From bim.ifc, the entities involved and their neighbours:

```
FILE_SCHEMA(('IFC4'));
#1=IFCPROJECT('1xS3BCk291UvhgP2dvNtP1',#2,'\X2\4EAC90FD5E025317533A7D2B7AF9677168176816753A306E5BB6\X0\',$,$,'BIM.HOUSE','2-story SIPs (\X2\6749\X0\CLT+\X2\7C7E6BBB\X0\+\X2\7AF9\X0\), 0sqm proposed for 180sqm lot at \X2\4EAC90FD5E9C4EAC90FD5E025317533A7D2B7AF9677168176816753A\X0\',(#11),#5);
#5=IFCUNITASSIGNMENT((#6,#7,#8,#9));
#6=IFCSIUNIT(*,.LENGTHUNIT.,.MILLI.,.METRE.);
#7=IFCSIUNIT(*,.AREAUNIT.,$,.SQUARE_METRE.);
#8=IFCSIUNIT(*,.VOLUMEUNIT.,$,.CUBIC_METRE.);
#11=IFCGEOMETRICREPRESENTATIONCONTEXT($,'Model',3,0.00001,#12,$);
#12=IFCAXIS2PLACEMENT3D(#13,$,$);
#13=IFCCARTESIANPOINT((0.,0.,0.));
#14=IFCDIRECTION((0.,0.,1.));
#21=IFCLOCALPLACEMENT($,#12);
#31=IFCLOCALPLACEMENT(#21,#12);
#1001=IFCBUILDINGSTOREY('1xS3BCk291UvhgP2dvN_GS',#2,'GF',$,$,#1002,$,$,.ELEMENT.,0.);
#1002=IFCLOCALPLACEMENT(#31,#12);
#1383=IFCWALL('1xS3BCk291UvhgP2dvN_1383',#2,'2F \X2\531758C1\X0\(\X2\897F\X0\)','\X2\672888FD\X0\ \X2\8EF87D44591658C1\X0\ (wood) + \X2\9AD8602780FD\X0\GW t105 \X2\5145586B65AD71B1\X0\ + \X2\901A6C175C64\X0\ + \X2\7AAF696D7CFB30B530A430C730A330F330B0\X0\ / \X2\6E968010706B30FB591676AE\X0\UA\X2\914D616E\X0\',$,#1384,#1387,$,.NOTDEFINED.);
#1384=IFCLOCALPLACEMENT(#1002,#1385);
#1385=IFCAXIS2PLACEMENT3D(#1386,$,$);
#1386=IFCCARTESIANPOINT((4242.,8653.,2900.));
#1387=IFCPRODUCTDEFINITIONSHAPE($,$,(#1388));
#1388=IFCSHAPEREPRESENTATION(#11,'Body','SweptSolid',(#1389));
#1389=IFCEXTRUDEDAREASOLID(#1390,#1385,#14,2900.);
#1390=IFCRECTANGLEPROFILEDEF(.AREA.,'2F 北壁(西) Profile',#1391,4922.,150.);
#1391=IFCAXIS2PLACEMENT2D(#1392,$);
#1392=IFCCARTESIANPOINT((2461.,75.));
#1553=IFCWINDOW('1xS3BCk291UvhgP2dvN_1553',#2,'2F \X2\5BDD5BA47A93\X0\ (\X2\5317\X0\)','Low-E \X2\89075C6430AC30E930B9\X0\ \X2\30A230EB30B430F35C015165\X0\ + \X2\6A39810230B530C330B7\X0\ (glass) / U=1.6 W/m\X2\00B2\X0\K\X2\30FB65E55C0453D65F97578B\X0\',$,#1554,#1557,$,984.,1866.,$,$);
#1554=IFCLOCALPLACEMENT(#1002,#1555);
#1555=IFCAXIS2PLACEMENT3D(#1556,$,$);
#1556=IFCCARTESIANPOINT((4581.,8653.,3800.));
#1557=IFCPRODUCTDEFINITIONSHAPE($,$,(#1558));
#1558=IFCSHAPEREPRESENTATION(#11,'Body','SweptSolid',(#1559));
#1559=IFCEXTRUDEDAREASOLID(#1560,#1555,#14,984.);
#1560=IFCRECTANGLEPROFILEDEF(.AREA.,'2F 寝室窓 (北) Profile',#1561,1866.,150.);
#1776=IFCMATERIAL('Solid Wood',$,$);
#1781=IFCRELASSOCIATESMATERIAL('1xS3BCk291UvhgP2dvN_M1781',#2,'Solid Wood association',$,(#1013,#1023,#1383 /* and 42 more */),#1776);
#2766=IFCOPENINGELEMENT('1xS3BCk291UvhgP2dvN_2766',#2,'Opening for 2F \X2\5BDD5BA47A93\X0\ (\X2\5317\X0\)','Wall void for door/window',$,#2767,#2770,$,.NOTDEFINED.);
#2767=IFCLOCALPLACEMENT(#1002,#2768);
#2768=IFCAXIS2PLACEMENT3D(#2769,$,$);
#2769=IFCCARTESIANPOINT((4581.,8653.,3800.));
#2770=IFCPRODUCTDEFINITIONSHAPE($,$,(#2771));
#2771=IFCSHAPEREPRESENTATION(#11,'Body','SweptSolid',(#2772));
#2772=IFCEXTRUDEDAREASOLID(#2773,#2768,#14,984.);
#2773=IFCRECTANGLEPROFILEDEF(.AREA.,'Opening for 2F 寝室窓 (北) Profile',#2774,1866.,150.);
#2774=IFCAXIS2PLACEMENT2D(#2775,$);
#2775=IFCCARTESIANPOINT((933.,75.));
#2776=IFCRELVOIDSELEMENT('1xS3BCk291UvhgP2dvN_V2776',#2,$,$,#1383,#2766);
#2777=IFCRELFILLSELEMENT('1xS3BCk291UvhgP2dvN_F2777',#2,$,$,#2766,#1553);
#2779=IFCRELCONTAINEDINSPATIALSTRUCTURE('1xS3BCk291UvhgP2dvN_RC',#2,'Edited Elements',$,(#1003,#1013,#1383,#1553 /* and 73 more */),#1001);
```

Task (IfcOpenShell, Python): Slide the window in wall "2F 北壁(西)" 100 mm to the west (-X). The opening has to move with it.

```python
import ifcopenshell
import ifcopenshell.api.geometry
import ifcopenshell.util.placement
import ifcopenshell.util.unit

model = ifcopenshell.open("bim.ifc")
unit_scale = ifcopenshell.util.unit.calculate_unit_scale(model)

window = model.by_guid("1xS3BCk291UvhgP2dvN_1553")
opening = window.FillsVoids[0].RelatingOpeningElement
wall = opening.VoidsElements[0].RelatingBuildingElement

wall_matrix = ifcopenshell.util.placement.get_local_placement(wall.ObjectPlacement)
shift = wall_matrix[:3, 0] * -0.1 / unit_scale
before = ifcopenshell.util.placement.get_local_placement(window.ObjectPlacement)[:3, 3].copy()

# The window is not placed relative to its opening, so move both.
for product in (opening, window):
    matrix = ifcopenshell.util.placement.get_local_placement(product.ObjectPlacement)
    matrix[:3, 3] += shift
    ifcopenshell.api.geometry.edit_object_placement(model, product=product, matrix=matrix, is_si=False)

after = ifcopenshell.util.placement.get_local_placement(window.ObjectPlacement)[:3, 3]
print("window moved by", (after - before).round(3) + 0.0)

model.write("bim_rev.ifc")
```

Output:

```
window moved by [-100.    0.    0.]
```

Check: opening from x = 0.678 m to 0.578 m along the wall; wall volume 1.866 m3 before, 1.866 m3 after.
